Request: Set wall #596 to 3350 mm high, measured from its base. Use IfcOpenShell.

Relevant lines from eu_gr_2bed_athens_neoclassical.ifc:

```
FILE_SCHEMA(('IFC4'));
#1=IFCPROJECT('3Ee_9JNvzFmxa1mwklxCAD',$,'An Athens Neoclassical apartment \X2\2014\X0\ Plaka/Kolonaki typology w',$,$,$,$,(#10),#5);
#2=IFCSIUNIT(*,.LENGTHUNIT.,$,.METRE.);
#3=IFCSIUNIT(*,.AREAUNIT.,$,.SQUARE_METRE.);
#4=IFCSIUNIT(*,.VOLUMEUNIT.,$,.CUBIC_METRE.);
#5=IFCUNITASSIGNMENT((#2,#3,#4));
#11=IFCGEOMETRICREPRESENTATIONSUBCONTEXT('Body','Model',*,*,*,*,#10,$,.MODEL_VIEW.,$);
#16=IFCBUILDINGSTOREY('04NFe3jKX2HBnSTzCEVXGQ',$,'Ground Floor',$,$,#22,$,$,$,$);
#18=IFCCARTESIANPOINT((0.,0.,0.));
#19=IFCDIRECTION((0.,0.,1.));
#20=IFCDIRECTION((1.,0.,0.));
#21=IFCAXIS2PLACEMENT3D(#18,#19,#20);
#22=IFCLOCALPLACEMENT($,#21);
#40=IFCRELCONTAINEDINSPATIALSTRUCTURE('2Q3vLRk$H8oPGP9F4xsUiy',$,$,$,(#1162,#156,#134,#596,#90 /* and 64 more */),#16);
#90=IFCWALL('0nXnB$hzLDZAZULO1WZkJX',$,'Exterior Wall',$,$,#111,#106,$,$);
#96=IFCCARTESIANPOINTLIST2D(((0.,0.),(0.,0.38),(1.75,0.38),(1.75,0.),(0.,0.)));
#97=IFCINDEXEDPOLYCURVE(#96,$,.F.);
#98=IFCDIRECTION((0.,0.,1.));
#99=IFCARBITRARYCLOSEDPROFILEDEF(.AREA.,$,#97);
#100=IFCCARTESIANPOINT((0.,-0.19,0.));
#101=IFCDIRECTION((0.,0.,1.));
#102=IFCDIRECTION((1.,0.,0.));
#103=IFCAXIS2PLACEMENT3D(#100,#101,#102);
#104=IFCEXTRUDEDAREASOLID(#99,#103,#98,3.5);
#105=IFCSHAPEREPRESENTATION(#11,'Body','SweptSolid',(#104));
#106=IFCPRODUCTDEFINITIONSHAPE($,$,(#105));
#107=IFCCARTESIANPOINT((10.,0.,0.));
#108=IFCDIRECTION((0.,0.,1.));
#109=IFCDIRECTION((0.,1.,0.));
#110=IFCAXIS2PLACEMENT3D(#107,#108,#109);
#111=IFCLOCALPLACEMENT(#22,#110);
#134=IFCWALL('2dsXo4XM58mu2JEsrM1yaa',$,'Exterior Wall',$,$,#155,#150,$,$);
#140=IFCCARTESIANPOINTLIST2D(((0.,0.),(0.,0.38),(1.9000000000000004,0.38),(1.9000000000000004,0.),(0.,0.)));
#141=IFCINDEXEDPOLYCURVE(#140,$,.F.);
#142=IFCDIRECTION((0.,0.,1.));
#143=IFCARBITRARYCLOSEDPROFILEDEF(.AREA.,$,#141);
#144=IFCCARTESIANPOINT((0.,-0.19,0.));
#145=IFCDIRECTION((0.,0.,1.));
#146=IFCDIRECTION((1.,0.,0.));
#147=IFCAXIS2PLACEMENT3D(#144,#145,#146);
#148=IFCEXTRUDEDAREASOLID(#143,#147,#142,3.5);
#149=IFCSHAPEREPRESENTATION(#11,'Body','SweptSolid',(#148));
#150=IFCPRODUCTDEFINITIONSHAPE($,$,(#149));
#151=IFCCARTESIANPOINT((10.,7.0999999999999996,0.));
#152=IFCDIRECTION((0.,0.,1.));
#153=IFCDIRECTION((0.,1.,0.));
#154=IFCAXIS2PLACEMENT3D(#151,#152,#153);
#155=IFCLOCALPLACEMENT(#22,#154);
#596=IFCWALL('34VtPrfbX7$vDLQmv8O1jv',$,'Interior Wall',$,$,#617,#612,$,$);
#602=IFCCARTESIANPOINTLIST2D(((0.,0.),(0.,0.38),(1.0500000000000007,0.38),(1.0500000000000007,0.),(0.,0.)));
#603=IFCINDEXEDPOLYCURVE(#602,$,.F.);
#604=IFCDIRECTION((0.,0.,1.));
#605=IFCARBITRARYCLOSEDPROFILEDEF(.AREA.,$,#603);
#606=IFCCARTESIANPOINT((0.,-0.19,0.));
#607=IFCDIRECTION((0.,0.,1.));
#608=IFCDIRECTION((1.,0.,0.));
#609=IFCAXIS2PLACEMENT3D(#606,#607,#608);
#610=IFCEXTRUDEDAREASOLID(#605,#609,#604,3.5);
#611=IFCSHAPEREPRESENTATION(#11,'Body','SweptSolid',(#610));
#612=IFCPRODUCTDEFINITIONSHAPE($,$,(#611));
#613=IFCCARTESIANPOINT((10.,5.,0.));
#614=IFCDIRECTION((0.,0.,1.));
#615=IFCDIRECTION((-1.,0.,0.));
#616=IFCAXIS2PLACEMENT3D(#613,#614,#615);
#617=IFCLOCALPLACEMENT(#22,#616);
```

```python
import ifcopenshell
import ifcopenshell.geom
import ifcopenshell.util.representation
import ifcopenshell.util.shape

model = ifcopenshell.open("eu_gr_2bed_athens_neoclassical.ifc")
settings = ifcopenshell.geom.settings()


def volume(element):
    """Net volume in cubic metres, openings subtracted."""
    shape = ifcopenshell.geom.create_shape(settings, element)
    return ifcopenshell.util.shape.get_volume(shape.geometry)


wall = model.by_guid("34VtPrfbX7$vDLQmv8O1jv")
before = volume(wall)

body = ifcopenshell.util.representation.get_representation(wall, "Model", "Body")
solid = body.Items[0]
old_height = solid.Depth
solid.Depth = 3.35
after = volume(wall)

print(f"height {old_height:g} -> {solid.Depth:g}, volume {before:.3f} -> {after:.3f} m3")

model.write("eu_gr_2bed_athens_neoclassical_rev.ifc")
```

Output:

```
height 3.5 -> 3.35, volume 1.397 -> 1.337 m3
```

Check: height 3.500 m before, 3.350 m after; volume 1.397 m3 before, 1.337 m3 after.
